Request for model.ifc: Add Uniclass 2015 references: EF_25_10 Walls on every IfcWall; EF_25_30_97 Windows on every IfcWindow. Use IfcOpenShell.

First a look at what the model holds.

```python
import ifcopenshell

model = ifcopenshell.open("model.ifc")
print(model.schema)
print("classifications:", [c.Name for c in model.by_type("IfcClassification")])
for ifc_class in ("IfcDoor", "IfcRoof", "IfcStair", "IfcWall", "IfcWindow"):
    print(ifc_class, len(model.by_type(ifc_class)))
```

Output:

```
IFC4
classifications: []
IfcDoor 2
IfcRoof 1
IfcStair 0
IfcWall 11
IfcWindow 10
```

```python
import ifcopenshell
import ifcopenshell.api.classification

model = ifcopenshell.open("model.ifc")

system = ifcopenshell.api.classification.add_classification(model, classification="Uniclass 2015")

codes = {
    "IfcWall": ("EF_25_10", "Walls"),
    "IfcWindow": ("EF_25_30_97", "Windows"),
}
for ifc_class, (code, name) in codes.items():
    products = model.by_type(ifc_class)
    ifcopenshell.api.classification.add_reference(
        model, products=products, classification=system, identification=code, name=name
    )
    print(code, len(products))

model.write("model_v2.ifc")
```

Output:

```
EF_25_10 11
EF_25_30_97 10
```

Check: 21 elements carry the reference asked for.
